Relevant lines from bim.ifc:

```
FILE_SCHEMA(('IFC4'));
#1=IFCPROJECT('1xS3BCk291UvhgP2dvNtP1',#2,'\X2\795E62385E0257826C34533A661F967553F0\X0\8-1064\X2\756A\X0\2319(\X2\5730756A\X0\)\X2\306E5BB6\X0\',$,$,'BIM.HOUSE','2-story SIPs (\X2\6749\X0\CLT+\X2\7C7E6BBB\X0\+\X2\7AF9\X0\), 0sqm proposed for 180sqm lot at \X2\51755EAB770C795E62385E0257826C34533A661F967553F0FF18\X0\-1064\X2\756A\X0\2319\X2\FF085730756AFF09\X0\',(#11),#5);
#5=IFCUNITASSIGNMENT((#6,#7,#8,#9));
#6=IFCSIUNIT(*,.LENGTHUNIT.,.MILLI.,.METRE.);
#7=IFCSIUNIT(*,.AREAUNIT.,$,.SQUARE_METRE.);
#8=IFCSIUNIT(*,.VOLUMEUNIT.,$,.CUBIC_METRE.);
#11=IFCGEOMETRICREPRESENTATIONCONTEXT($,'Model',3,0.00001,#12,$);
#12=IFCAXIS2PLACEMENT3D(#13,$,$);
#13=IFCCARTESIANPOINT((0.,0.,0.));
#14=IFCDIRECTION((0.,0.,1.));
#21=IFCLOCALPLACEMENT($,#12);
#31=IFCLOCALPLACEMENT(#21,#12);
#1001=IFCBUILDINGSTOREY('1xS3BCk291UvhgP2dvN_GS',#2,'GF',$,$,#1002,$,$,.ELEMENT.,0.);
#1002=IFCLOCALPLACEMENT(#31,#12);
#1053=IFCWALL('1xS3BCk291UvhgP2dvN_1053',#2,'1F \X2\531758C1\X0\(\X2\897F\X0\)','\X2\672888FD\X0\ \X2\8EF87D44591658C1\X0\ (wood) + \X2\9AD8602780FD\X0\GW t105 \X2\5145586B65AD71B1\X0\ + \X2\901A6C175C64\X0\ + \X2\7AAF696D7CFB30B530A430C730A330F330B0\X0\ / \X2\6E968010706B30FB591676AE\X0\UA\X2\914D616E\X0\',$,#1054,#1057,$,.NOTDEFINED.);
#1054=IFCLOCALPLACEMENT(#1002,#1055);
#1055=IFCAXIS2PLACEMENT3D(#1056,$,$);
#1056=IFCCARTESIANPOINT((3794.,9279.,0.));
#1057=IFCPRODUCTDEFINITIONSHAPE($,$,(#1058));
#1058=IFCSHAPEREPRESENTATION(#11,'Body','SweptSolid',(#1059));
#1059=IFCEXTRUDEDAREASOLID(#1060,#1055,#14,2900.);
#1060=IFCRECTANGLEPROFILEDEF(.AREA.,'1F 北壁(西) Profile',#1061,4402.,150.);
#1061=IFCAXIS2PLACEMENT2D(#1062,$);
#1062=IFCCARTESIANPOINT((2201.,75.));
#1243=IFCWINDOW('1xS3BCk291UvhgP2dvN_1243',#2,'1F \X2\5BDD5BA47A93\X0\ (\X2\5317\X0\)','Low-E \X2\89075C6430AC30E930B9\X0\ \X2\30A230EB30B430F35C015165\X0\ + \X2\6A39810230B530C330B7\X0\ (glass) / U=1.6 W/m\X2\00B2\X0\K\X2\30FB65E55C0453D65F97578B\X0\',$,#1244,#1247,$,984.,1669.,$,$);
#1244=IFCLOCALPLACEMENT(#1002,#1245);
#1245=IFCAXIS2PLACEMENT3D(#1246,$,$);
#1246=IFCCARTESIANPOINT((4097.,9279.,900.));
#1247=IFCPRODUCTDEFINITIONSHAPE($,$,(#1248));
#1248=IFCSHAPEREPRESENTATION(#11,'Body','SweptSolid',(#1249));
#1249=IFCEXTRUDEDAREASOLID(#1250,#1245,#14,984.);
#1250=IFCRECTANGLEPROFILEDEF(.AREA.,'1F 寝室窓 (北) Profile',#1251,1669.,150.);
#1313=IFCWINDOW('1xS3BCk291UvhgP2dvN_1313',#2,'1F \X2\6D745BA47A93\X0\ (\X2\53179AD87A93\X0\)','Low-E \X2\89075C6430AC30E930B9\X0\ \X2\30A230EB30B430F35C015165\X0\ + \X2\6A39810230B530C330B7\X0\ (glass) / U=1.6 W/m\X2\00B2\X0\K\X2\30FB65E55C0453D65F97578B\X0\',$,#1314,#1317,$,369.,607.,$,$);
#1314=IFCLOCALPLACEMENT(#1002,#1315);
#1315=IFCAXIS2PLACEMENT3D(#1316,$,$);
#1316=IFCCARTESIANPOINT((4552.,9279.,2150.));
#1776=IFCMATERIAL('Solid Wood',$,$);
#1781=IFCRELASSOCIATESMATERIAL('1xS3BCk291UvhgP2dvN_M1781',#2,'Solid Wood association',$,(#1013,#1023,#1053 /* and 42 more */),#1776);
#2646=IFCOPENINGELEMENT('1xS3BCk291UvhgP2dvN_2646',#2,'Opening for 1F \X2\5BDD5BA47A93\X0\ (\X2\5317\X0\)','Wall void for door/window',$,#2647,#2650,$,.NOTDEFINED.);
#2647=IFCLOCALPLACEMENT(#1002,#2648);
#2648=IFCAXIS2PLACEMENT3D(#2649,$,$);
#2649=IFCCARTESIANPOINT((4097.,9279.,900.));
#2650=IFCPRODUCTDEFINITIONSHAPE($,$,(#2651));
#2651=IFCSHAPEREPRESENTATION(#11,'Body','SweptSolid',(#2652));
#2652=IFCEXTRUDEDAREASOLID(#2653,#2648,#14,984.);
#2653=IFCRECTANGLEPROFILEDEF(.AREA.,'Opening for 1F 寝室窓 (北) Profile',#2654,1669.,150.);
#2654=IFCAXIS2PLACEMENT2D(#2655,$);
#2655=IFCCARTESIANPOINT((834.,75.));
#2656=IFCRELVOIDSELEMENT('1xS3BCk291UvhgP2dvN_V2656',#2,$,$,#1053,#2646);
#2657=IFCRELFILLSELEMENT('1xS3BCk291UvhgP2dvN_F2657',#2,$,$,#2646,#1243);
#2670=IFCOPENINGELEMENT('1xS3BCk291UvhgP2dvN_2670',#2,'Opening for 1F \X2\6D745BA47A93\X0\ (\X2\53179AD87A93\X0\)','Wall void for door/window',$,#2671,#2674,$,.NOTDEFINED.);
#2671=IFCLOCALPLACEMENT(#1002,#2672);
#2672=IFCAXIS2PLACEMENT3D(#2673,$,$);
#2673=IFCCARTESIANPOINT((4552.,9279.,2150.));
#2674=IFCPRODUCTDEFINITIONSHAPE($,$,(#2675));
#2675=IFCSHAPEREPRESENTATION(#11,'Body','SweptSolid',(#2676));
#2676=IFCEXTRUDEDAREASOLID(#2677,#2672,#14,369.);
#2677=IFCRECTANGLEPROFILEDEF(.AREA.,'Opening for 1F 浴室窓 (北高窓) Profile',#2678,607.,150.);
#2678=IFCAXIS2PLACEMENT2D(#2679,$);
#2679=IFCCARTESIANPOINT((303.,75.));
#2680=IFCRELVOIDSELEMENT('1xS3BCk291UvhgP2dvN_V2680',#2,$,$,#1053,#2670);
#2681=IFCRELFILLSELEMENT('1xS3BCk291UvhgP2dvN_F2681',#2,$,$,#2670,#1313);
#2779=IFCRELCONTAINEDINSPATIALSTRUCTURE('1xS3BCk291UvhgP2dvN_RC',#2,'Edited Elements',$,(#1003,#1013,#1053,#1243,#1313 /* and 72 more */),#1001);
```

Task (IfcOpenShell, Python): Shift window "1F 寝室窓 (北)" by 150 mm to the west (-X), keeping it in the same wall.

```python
import ifcopenshell
import ifcopenshell.api.geometry
import ifcopenshell.util.placement
import ifcopenshell.util.unit

model = ifcopenshell.open("bim.ifc")
unit_scale = ifcopenshell.util.unit.calculate_unit_scale(model)

window = model.by_guid("1xS3BCk291UvhgP2dvN_1243")
opening = window.FillsVoids[0].RelatingOpeningElement
wall = opening.VoidsElements[0].RelatingBuildingElement

wall_matrix = ifcopenshell.util.placement.get_local_placement(wall.ObjectPlacement)
shift = wall_matrix[:3, 0] * -0.15 / unit_scale
before = ifcopenshell.util.placement.get_local_placement(window.ObjectPlacement)[:3, 3].copy()

# The window is not placed relative to its opening, so move both.
for product in (opening, window):
    matrix = ifcopenshell.util.placement.get_local_placement(product.ObjectPlacement)
    matrix[:3, 3] += shift
    ifcopenshell.api.geometry.edit_object_placement(model, product=product, matrix=matrix, is_si=False)

after = ifcopenshell.util.placement.get_local_placement(window.ObjectPlacement)[:3, 3]
print("window moved by", (after - before).round(3) + 0.0)

model.write("bim_v2.ifc")
```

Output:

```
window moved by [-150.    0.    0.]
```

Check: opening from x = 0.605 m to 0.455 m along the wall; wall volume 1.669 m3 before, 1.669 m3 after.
